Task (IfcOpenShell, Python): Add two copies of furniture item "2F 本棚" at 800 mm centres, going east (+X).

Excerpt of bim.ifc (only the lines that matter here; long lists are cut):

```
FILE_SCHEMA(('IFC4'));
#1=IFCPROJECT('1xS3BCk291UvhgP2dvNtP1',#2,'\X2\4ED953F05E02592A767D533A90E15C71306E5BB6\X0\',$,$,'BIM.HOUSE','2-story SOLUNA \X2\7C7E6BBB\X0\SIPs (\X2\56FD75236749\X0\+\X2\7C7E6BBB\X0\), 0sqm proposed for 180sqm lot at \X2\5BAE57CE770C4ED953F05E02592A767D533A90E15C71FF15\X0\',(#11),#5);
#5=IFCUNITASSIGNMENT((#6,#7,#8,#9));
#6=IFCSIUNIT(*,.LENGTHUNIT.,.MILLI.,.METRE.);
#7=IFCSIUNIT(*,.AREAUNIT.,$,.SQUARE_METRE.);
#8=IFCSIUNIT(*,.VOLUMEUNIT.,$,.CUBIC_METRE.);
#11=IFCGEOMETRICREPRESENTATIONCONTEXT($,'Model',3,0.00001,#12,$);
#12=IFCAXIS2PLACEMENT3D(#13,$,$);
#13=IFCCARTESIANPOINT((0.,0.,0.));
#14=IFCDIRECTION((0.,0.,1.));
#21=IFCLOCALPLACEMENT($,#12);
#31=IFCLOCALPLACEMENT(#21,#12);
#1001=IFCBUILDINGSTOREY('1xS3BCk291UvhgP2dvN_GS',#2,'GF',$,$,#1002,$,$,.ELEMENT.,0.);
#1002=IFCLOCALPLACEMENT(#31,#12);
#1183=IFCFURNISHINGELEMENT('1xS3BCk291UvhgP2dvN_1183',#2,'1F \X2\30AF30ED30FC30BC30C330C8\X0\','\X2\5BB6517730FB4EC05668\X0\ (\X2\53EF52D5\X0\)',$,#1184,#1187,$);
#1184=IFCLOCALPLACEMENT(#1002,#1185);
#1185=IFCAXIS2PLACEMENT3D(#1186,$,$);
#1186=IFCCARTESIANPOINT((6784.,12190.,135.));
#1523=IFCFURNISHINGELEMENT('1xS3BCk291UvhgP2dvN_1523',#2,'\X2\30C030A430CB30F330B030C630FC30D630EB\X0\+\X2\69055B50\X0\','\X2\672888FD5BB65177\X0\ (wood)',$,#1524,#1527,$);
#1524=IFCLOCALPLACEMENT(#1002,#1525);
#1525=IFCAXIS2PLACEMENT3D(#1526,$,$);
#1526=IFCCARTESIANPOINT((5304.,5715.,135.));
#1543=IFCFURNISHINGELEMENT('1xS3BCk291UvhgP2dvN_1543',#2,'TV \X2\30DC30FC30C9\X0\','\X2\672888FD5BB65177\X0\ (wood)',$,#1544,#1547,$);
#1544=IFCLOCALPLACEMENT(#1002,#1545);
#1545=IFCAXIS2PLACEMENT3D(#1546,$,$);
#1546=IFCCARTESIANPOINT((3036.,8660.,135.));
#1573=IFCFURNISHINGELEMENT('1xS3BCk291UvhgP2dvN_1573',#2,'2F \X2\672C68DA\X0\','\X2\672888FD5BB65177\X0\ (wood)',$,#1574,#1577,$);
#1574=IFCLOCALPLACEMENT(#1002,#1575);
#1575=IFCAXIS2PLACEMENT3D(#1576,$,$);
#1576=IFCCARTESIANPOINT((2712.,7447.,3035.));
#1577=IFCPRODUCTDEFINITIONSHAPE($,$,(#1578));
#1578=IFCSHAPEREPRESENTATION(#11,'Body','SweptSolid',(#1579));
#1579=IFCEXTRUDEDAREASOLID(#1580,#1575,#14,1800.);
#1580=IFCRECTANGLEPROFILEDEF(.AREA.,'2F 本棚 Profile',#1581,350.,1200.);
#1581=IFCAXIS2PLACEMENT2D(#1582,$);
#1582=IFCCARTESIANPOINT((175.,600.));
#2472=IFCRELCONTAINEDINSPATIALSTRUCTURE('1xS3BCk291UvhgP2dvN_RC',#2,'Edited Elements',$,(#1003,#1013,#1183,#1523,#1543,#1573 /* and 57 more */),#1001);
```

```python
import numpy as np
import ifcopenshell
import ifcopenshell.api.geometry
import ifcopenshell.api.root
import ifcopenshell.util.element
import ifcopenshell.util.placement
import ifcopenshell.util.unit

model = ifcopenshell.open("bim.ifc")
unit_scale = ifcopenshell.util.unit.calculate_unit_scale(model)


def reuse_history(source, copy):
    """copy_class also copies each property set's owner history, people and application; keep the originals."""
    for rel in copy.IsDefinedBy:
        if rel.is_a("IfcRelDefinesByProperties") and (history := rel.RelatingPropertyDefinition.OwnerHistory):
            rel.RelatingPropertyDefinition.OwnerHistory = source.OwnerHistory
            ifcopenshell.util.element.remove_deep2(model, history)


source = model.by_guid("1xS3BCk291UvhgP2dvN_1573")
base = ifcopenshell.util.placement.get_local_placement(source.ObjectPlacement)
step = np.array([1.0, 0.0, 0.0]) * 0.8 / unit_scale

for i in range(1, 3):
    copy = ifcopenshell.api.root.copy_class(model, product=source)
    copy.Representation = ifcopenshell.util.element.copy_deep(
        model, source.Representation, exclude=["IfcGeometricRepresentationContext", "IfcRepresentationMap"]
    )
    reuse_history(source, copy)
    matrix = base.copy()
    matrix[:3, 3] += i * step
    print("added at", matrix[:3, 3].round(3) + 0.0)
    ifcopenshell.api.geometry.edit_object_placement(model, product=copy, matrix=matrix, is_si=False)

model.write("bim-out.ifc")
```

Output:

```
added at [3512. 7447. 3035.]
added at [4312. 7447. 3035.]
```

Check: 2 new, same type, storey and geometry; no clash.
